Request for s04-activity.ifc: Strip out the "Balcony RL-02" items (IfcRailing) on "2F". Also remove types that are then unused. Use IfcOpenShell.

First a look at what the model holds.

```python
import ifcopenshell
import ifcopenshell.util.element

model = ifcopenshell.open("s04-activity.ifc")
print(model.schema)
storey = next(s for s in model.by_type("IfcBuildingStorey") if s.Name == "2F")
railings = [e for e in ifcopenshell.util.element.get_decomposition(storey) if e.is_a("IfcRailing")]
seen = {}
for e in railings:
    element_type = ifcopenshell.util.element.get_type(e)
    name = element_type.Name if element_type not in (None, e) else None
    seen[name] = seen.get(name, 0) + 1
for name, count in sorted(seen.items(), key=str):
    print(count, "x", name)
```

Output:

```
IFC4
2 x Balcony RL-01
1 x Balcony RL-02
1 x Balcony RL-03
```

```python
import ifcopenshell
import ifcopenshell.api.root
import ifcopenshell.util.element

model = ifcopenshell.open("s04-activity.ifc")

storey = next(s for s in model.by_type("IfcBuildingStorey") if s.Name == "2F")
railings = [e for e in ifcopenshell.util.element.get_decomposition(storey) if e.is_a("IfcRailing")]
targets = [e for e in railings if (t := ifcopenshell.util.element.get_type(e)) not in (None, e) and t.Name == "Balcony RL-02"]
types = {ifcopenshell.util.element.get_type(e) for e in targets} - {None, *targets}

for e in targets:
    ifcopenshell.api.root.remove_product(model, product=e)
print(len(targets), "removed")

unused = [t for t in types if not ifcopenshell.util.element.get_types(t)]
for t in unused:
    ifcopenshell.api.root.remove_product(model, product=t)
print(len(unused), "unused types removed")

model.write("s04-activity_rev.ifc")
```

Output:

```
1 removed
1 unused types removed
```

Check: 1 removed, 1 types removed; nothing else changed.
